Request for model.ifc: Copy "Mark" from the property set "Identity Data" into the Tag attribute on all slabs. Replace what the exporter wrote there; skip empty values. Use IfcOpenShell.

First a look at what the model holds.

```python
import ifcopenshell
import ifcopenshell.util.element

model = ifcopenshell.open("model.ifc")
print(model.schema)
slabs = model.by_type("IfcSlab")
print(len(slabs), "slabs")
for e in slabs[:8]:
    source = ifcopenshell.util.element.get_pset(e, "Identity Data", "Mark")
    target = e.Tag
    print(e.id(), repr(source), repr(target), sep=" | ")
```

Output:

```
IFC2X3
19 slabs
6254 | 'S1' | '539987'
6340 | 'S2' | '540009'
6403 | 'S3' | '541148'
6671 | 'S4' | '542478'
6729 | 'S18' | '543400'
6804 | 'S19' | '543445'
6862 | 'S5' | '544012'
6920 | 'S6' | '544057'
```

```python
import ifcopenshell
import ifcopenshell.util.element

model = ifcopenshell.open("model.ifc")

count = 0
for e in model.by_type("IfcSlab"):
    value = ifcopenshell.util.element.get_pset(e, "Identity Data", "Mark")
    current = e.Tag
    if not value or not value.strip() or current == value:
        continue
    e.Tag = value
    count += 1

print(count, "slabs updated")

model.write("model_edited.ifc")
```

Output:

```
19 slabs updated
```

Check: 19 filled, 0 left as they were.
